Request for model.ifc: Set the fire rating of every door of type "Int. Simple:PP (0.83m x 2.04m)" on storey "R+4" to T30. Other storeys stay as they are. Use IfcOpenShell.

First a look at what the model holds.

```python
import ifcopenshell
import ifcopenshell.util.element

model = ifcopenshell.open("model.ifc")
print(model.schema)
storey = next(s for s in model.by_type("IfcBuildingStorey") if s.Name == "R+4")
doors = [e for e in ifcopenshell.util.element.get_decomposition(storey) if e.is_a("IfcDoor")]
seen = {}
for e in doors:
    element_type = ifcopenshell.util.element.get_type(e)
    key = (element_type.Name if element_type != e and element_type else None, ifcopenshell.util.element.get_pset(e, "Pset_DoorCommon", "FireRating"))
    seen[key] = seen.get(key, 0) + 1
for (name, value), count in sorted(seen.items(), key=str):
    print(count, "x", name, "|", value)
```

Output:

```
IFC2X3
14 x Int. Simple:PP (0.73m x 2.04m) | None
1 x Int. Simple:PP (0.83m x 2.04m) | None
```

```python
import ifcopenshell
import ifcopenshell.api.pset
import ifcopenshell.util.element

model = ifcopenshell.open("model.ifc")

storey = next(s for s in model.by_type("IfcBuildingStorey") if s.Name == "R+4")
doors = [e for e in ifcopenshell.util.element.get_decomposition(storey) if e.is_a("IfcDoor")]

count = 0
for e in doors:
    element_type = ifcopenshell.util.element.get_type(e)
    if element_type in (None, e) or element_type.Name != "Int. Simple:PP (0.83m x 2.04m)":
        continue
    # add_pset returns the element's existing set when there is one.
    pset = ifcopenshell.api.pset.add_pset(model, product=e, name="Pset_DoorCommon")
    ifcopenshell.api.pset.edit_pset(model, pset=pset, properties={"FireRating": "T30"})
    count += 1

print(count, "doors updated")

model.write("model_edited.ifc")
```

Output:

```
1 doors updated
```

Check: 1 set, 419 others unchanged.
